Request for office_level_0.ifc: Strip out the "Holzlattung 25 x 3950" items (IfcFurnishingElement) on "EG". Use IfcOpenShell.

First a look at what the model holds.

```python
import ifcopenshell
import ifcopenshell.util.element

model = ifcopenshell.open("office_level_0.ifc")
print(model.schema)
storey = next(s for s in model.by_type("IfcBuildingStorey") if s.Name == "EG")
furniture = [e for e in ifcopenshell.util.element.get_decomposition(storey) if e.is_a("IfcFurnishingElement")]
seen = {}
for e in furniture:
    element_type = ifcopenshell.util.element.get_type(e)
    name = element_type.Name if element_type not in (None, e) else None
    seen[name] = seen.get(name, 0) + 1
for name, count in sorted(seen.items(), key=str):
    print(count, "x", name)
```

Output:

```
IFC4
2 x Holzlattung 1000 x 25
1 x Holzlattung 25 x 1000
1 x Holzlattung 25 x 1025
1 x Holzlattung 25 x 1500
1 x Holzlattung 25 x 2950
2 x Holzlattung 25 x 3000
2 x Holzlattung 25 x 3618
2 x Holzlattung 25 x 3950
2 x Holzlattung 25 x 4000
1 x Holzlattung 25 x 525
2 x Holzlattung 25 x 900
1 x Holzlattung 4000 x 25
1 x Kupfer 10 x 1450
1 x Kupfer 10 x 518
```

```python
import ifcopenshell
import ifcopenshell.api.root
import ifcopenshell.util.element

model = ifcopenshell.open("office_level_0.ifc")

storey = next(s for s in model.by_type("IfcBuildingStorey") if s.Name == "EG")
furniture = [e for e in ifcopenshell.util.element.get_decomposition(storey) if e.is_a("IfcFurnishingElement")]
targets = [e for e in furniture if (t := ifcopenshell.util.element.get_type(e)) not in (None, e) and t.Name == "Holzlattung 25 x 3950"]

for e in targets:
    ifcopenshell.api.root.remove_product(model, product=e)
print(len(targets), "removed")

model.write("office_level_0_rev.ifc")
```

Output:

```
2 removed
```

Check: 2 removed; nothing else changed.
